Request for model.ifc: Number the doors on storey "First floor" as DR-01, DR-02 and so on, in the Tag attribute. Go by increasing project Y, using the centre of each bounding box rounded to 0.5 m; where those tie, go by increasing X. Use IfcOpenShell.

First a look at what the model holds.

```python
import ifcopenshell
import ifcopenshell.util.element
import ifcopenshell.util.placement

model = ifcopenshell.open("model.ifc")
print(model.schema)
storey = next(s for s in model.by_type("IfcBuildingStorey") if s.Name == "First floor")
doors = [e for e in ifcopenshell.util.element.get_decomposition(storey) if e.is_a("IfcDoor")]
for e in sorted(doors, key=lambda e: e.id()):
    origin = ifcopenshell.util.placement.get_local_placement(e.ObjectPlacement)[:3, 3]
    print(e.id(), e.Tag, e.Name, origin.round(2) + 0.0, sep=" | ")
```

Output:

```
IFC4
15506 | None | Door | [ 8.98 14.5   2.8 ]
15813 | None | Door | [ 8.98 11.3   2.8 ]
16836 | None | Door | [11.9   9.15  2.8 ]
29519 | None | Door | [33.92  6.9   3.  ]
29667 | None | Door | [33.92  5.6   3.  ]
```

```python
import ifcopenshell
import ifcopenshell.geom
import ifcopenshell.util.element
import ifcopenshell.util.shape

model = ifcopenshell.open("model.ifc")
settings = ifcopenshell.geom.settings()
settings.set("use-world-coords", True)


def centre(element):
    shape = ifcopenshell.geom.create_shape(settings, element)
    return ifcopenshell.util.shape.get_bbox_centroid(shape.geometry)


storey = next(s for s in model.by_type("IfcBuildingStorey") if s.Name == "First floor")
doors = [e for e in ifcopenshell.util.element.get_decomposition(storey) if e.is_a("IfcDoor")]

# Insertion points can sit at a corner or the storey origin, so sort by the geometry (in metres).
centres = {e: centre(e) for e in doors}
doors.sort(key=lambda e: (round(centres[e][1] / 0.5), centres[e][0]))

for i, e in enumerate(doors, start=1):
    number = f"DR-{i:02d}"
    e.Tag = number
    print(e.id(), number)

model.write("model_v2.ifc")
```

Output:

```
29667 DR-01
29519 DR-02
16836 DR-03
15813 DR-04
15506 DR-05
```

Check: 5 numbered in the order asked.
